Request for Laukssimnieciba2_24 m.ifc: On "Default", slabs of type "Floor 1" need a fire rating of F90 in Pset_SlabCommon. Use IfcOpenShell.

First a look at what the model holds.

```python
import ifcopenshell
import ifcopenshell.util.element

model = ifcopenshell.open("Laukssimnieciba2_24 m.ifc")
print(model.schema)
storey = next(s for s in model.by_type("IfcBuildingStorey") if s.Name == "Default")
slabs = [e for e in ifcopenshell.util.element.get_decomposition(storey) if e.is_a("IfcSlab")]
seen = {}
for e in slabs:
    element_type = ifcopenshell.util.element.get_type(e)
    key = (element_type.Name if element_type != e and element_type else None, ifcopenshell.util.element.get_pset(e, "Pset_SlabCommon", "FireRating"))
    seen[key] = seen.get(key, 0) + 1
for (name, value), count in sorted(seen.items(), key=str):
    print(count, "x", name, "|", value)
```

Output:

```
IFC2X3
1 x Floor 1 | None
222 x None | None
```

```python
import ifcopenshell
import ifcopenshell.api.pset
import ifcopenshell.util.element

model = ifcopenshell.open("Laukssimnieciba2_24 m.ifc")

storey = next(s for s in model.by_type("IfcBuildingStorey") if s.Name == "Default")
slabs = [e for e in ifcopenshell.util.element.get_decomposition(storey) if e.is_a("IfcSlab")]

count = 0
for e in slabs:
    element_type = ifcopenshell.util.element.get_type(e)
    if element_type in (None, e) or element_type.Name != "Floor 1":
        continue
    # add_pset returns the element's existing set when there is one.
    pset = ifcopenshell.api.pset.add_pset(model, product=e, name="Pset_SlabCommon")
    ifcopenshell.api.pset.edit_pset(model, pset=pset, properties={"FireRating": "F90"})
    count += 1

print(count, "slabs updated")

model.write("Laukssimnieciba2_24 m_updated.ifc")
```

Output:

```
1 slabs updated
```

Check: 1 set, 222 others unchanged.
